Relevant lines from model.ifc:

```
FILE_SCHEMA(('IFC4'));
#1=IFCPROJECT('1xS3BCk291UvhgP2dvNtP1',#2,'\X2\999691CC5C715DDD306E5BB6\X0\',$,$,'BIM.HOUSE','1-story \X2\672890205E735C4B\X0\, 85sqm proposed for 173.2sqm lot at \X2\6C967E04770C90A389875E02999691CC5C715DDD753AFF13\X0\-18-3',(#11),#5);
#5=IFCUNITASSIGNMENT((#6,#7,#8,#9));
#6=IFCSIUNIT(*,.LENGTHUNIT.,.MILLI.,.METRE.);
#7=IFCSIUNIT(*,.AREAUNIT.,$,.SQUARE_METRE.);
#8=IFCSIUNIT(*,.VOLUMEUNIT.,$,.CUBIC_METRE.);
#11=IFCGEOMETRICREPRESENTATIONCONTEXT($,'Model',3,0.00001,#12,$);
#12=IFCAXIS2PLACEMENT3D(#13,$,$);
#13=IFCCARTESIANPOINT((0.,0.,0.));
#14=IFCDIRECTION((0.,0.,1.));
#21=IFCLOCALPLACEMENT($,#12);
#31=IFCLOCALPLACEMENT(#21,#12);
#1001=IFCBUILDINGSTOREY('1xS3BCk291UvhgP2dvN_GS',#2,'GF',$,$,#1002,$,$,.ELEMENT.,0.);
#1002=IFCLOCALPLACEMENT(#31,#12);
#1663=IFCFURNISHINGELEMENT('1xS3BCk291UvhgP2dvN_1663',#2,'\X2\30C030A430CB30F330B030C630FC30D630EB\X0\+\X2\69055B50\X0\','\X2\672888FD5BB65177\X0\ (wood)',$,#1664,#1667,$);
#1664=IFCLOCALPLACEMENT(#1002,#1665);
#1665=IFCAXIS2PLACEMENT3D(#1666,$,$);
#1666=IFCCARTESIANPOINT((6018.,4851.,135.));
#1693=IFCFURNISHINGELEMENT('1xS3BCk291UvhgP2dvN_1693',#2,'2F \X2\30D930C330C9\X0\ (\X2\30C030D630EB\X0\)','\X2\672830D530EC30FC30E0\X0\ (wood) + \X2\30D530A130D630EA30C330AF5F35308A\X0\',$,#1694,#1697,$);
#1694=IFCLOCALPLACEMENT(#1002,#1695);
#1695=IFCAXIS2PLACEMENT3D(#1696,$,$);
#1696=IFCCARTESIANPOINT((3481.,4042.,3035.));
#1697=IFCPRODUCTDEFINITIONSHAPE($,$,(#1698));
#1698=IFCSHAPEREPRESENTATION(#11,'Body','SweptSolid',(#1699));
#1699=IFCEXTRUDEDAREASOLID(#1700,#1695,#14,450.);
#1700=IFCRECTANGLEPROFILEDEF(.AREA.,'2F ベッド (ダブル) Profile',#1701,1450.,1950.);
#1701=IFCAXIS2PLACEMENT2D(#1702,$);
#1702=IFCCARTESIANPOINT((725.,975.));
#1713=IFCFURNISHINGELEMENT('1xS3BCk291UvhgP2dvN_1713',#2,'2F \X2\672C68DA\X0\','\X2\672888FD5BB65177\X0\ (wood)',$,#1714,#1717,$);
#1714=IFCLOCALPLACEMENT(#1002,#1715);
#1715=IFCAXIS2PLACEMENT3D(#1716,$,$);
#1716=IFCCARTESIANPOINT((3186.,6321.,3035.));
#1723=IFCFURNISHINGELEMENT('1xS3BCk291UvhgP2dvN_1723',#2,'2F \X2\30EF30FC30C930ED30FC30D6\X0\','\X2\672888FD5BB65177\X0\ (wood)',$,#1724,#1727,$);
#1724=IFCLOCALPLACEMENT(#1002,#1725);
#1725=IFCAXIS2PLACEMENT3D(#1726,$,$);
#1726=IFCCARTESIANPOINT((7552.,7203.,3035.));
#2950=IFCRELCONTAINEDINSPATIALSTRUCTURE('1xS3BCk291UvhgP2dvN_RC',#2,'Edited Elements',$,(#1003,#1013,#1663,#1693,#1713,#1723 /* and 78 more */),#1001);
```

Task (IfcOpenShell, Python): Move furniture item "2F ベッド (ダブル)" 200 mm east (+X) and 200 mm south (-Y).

```python
import ifcopenshell
import ifcopenshell.api.geometry
import ifcopenshell.util.placement
import ifcopenshell.util.unit

model = ifcopenshell.open("model.ifc")
unit_scale = ifcopenshell.util.unit.calculate_unit_scale(model)

item = model.by_guid("1xS3BCk291UvhgP2dvN_1693")
matrix = ifcopenshell.util.placement.get_local_placement(item.ObjectPlacement)
matrix[0, 3] += 0.2 / unit_scale
matrix[1, 3] -= 0.2 / unit_scale
ifcopenshell.api.geometry.edit_object_placement(model, product=item, matrix=matrix, is_si=False)

print(ifcopenshell.util.placement.get_local_placement(item.ObjectPlacement).round(3) + 0.0)

model.write("model_v2.ifc")
```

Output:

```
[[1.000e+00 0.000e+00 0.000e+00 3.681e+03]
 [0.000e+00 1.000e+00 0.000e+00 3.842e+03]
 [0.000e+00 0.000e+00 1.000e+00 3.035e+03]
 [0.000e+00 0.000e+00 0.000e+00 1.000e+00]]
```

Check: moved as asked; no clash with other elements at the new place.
